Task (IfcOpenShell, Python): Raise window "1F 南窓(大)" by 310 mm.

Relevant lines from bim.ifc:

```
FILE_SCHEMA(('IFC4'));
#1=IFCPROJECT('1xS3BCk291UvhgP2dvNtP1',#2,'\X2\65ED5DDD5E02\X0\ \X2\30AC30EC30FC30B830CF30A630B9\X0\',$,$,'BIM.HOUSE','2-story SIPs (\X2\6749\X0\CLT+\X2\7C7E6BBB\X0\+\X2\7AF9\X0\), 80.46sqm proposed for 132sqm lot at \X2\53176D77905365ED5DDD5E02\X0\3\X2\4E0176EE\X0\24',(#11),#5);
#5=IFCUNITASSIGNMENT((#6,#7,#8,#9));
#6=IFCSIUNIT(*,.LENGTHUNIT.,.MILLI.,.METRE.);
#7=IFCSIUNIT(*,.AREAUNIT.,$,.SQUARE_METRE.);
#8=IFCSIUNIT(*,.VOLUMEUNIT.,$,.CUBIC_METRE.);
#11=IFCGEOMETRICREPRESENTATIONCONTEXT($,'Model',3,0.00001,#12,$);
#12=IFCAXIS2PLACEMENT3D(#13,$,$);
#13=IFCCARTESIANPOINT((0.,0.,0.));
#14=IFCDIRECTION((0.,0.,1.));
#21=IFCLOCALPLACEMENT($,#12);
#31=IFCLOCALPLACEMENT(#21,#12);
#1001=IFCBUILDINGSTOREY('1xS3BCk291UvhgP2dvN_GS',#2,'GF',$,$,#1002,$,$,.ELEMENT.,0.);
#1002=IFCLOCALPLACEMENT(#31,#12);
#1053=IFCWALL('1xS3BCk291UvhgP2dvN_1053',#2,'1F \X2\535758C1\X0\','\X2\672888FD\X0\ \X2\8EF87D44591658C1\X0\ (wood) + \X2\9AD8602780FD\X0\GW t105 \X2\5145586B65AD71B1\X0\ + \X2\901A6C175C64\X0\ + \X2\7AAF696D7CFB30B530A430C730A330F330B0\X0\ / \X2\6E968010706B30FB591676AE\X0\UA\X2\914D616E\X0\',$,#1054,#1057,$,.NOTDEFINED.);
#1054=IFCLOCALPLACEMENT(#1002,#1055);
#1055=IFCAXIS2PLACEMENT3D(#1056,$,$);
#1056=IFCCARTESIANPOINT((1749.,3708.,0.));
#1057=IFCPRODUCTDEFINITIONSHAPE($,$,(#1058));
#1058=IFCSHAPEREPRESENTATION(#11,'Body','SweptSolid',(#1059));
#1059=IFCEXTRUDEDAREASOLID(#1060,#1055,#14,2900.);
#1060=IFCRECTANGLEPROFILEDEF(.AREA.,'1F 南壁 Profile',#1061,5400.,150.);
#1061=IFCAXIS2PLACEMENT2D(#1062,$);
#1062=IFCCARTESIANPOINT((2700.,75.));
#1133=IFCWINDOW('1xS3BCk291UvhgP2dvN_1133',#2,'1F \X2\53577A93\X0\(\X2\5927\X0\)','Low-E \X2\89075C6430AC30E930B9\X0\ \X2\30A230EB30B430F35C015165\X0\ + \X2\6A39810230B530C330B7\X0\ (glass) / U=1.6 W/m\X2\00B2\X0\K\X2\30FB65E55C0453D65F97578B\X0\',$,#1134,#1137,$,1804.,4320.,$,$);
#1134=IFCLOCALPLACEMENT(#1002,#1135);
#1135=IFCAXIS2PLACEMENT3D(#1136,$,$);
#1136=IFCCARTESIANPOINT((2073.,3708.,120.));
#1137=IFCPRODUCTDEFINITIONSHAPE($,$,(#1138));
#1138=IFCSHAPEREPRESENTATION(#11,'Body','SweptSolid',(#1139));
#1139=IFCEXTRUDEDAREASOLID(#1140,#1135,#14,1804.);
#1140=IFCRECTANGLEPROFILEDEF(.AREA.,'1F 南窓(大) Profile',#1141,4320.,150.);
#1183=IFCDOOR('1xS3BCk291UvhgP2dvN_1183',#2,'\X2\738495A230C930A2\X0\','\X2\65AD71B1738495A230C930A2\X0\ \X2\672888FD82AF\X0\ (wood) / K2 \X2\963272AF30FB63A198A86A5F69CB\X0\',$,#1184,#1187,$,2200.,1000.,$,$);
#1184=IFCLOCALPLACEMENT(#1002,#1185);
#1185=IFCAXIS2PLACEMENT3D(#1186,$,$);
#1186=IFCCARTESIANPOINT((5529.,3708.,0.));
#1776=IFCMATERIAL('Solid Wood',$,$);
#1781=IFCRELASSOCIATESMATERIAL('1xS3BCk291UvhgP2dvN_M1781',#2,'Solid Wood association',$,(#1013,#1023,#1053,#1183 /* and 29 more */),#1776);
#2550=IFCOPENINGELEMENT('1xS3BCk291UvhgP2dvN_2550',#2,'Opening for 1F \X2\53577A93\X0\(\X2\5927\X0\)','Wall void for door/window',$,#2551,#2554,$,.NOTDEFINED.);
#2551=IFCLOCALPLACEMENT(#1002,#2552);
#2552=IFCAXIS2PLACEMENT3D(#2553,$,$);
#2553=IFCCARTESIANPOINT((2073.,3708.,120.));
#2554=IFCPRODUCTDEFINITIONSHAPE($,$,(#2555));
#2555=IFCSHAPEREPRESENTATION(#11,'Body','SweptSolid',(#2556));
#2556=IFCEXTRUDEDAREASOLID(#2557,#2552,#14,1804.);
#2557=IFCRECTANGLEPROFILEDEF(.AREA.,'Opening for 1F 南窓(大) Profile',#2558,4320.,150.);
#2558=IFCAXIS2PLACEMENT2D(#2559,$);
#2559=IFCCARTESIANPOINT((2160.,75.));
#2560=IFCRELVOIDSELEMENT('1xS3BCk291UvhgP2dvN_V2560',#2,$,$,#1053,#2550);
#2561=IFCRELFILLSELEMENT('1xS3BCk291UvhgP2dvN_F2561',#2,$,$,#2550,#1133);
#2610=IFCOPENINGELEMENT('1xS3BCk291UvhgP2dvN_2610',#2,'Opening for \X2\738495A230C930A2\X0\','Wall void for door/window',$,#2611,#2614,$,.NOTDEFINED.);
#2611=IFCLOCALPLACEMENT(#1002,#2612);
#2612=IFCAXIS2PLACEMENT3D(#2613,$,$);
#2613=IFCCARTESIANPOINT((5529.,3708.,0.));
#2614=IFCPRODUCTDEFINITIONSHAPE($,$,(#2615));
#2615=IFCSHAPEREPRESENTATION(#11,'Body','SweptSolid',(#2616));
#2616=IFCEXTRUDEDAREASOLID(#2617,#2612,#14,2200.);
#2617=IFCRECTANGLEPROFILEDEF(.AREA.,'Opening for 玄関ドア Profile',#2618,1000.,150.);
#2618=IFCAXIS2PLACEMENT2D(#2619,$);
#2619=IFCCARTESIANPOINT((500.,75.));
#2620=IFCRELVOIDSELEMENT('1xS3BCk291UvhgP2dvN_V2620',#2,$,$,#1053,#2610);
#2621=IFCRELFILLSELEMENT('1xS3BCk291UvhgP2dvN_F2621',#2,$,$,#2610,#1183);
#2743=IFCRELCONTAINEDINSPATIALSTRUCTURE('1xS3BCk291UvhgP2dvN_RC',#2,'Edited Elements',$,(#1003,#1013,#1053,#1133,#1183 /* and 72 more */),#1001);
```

```python
import numpy as np
import ifcopenshell
import ifcopenshell.api.geometry
import ifcopenshell.util.placement
import ifcopenshell.util.unit

model = ifcopenshell.open("bim.ifc")
unit_scale = ifcopenshell.util.unit.calculate_unit_scale(model)

window = model.by_guid("1xS3BCk291UvhgP2dvN_1133")
opening = window.FillsVoids[0].RelatingOpeningElement
dz = 0.31 / unit_scale

shift = np.array([0.0, 0.0, dz])
# The window is not placed relative to its opening, so move both.
for product in (opening, window):
    matrix = ifcopenshell.util.placement.get_local_placement(product.ObjectPlacement)
    matrix[:3, 3] += shift
    ifcopenshell.api.geometry.edit_object_placement(model, product=product, matrix=matrix, is_si=False)

print(f"moved by {dz * unit_scale:+.3f} m")

model.write("bim_edited.ifc")
```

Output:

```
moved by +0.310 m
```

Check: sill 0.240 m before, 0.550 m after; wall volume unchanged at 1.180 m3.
